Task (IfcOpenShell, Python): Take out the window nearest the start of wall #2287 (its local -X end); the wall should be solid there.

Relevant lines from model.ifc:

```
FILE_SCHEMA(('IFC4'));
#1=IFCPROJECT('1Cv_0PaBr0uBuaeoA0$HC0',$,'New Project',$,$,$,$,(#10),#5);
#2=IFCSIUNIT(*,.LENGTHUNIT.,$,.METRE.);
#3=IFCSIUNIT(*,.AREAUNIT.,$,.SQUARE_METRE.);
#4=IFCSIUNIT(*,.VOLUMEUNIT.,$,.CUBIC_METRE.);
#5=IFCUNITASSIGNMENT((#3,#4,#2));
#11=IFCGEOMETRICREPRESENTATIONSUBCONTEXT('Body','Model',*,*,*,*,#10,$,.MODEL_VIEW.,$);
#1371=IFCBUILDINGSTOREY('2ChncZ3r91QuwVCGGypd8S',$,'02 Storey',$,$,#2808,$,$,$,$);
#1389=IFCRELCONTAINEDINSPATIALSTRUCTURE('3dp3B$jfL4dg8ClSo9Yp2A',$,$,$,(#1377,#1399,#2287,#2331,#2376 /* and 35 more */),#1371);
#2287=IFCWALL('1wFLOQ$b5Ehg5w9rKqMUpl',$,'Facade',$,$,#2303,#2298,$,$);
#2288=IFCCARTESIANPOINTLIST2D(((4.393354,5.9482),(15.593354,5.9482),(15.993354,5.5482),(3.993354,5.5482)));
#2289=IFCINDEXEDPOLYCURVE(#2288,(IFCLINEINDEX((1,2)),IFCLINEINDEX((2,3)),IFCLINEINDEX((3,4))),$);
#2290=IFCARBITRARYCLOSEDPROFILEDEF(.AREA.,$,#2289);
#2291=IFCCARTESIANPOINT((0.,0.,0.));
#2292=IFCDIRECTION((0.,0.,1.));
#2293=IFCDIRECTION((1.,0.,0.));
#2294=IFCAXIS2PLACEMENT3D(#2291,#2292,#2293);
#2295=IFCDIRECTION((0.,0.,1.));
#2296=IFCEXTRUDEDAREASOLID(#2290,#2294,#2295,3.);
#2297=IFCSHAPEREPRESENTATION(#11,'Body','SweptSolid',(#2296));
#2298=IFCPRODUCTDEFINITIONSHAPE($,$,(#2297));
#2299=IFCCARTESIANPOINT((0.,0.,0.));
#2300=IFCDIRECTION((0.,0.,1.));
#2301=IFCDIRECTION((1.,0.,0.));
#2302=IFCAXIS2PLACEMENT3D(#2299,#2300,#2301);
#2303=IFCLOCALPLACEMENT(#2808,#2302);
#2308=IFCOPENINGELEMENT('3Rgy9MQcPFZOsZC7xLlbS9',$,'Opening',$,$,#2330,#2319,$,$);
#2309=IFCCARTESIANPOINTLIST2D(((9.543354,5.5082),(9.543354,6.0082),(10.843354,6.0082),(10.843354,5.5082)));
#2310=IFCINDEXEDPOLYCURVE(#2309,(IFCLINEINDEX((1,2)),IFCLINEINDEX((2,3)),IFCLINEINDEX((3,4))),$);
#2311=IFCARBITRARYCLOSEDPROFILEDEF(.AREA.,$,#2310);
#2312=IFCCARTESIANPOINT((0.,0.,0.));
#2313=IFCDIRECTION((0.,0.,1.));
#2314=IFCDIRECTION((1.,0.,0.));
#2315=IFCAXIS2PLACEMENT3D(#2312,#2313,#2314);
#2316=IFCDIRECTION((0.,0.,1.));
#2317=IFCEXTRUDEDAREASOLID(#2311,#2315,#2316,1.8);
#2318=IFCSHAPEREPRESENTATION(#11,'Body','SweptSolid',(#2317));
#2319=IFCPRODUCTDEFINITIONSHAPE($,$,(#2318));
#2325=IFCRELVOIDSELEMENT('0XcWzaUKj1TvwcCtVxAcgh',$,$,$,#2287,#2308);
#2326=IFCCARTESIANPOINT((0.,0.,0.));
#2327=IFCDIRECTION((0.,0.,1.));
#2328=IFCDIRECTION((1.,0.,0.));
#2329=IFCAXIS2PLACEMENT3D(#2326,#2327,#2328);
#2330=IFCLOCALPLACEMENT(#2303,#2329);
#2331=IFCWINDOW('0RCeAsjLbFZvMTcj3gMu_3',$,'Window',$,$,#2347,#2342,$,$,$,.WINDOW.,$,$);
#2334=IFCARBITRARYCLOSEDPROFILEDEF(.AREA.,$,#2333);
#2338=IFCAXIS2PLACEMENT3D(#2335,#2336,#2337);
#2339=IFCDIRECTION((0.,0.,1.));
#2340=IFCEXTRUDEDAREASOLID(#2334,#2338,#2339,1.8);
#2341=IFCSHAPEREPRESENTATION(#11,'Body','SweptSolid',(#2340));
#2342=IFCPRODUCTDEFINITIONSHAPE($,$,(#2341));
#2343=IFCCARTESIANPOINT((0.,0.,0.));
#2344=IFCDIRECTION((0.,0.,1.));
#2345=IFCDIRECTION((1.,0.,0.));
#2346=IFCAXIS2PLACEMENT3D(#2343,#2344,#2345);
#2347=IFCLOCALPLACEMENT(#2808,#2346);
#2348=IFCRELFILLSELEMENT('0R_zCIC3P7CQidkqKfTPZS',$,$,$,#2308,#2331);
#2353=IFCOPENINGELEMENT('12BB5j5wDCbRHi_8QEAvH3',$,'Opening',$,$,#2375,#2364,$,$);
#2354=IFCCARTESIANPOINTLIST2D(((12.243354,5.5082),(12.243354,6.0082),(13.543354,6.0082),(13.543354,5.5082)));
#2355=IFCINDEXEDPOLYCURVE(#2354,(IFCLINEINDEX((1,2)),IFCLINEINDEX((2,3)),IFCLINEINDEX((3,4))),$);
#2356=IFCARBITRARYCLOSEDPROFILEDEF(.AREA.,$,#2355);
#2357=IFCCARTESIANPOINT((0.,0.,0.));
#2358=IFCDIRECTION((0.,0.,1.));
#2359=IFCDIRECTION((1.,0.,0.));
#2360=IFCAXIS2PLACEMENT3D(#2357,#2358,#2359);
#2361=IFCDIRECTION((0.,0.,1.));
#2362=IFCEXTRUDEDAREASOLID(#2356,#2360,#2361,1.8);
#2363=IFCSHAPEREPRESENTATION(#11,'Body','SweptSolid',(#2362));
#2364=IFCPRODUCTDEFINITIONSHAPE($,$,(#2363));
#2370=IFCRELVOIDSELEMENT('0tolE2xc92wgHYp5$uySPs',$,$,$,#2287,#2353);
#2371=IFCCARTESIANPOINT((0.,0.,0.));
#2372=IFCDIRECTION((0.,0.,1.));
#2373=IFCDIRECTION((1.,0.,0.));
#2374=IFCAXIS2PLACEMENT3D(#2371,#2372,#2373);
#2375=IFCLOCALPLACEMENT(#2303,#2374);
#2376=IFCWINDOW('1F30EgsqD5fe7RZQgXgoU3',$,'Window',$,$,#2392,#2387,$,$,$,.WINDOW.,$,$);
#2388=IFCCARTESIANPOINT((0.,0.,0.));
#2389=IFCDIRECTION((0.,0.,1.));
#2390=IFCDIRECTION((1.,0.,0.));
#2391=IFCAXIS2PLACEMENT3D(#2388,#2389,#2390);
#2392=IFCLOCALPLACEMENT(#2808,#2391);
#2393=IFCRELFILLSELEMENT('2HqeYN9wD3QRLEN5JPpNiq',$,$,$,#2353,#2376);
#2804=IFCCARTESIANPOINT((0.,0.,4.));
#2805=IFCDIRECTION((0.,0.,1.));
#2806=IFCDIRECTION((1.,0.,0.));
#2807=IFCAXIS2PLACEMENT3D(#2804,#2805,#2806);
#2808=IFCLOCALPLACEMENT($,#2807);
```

```python
import ifcopenshell
import ifcopenshell.api.feature
import ifcopenshell.api.root
import ifcopenshell.geom
import ifcopenshell.util.shape

model = ifcopenshell.open("model.ifc")
settings = ifcopenshell.geom.settings()


def volume(element):
    """Net volume in cubic metres, openings subtracted."""
    shape = ifcopenshell.geom.create_shape(settings, element)
    return ifcopenshell.util.shape.get_volume(shape.geometry)


window = model.by_guid("0RCeAsjLbFZvMTcj3gMu_3")
opening = window.FillsVoids[0].RelatingOpeningElement
wall = opening.VoidsElements[0].RelatingBuildingElement
before = volume(wall)

ifcopenshell.api.root.remove_product(model, product=window)
ifcopenshell.api.feature.remove_feature(model, feature=opening)

after = volume(wall)

print(f"wall volume {before:.3f} -> {after:.3f} m3")

model.write("model_rev.ifc")
```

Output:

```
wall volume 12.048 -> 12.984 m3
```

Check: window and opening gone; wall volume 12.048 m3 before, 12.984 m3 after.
